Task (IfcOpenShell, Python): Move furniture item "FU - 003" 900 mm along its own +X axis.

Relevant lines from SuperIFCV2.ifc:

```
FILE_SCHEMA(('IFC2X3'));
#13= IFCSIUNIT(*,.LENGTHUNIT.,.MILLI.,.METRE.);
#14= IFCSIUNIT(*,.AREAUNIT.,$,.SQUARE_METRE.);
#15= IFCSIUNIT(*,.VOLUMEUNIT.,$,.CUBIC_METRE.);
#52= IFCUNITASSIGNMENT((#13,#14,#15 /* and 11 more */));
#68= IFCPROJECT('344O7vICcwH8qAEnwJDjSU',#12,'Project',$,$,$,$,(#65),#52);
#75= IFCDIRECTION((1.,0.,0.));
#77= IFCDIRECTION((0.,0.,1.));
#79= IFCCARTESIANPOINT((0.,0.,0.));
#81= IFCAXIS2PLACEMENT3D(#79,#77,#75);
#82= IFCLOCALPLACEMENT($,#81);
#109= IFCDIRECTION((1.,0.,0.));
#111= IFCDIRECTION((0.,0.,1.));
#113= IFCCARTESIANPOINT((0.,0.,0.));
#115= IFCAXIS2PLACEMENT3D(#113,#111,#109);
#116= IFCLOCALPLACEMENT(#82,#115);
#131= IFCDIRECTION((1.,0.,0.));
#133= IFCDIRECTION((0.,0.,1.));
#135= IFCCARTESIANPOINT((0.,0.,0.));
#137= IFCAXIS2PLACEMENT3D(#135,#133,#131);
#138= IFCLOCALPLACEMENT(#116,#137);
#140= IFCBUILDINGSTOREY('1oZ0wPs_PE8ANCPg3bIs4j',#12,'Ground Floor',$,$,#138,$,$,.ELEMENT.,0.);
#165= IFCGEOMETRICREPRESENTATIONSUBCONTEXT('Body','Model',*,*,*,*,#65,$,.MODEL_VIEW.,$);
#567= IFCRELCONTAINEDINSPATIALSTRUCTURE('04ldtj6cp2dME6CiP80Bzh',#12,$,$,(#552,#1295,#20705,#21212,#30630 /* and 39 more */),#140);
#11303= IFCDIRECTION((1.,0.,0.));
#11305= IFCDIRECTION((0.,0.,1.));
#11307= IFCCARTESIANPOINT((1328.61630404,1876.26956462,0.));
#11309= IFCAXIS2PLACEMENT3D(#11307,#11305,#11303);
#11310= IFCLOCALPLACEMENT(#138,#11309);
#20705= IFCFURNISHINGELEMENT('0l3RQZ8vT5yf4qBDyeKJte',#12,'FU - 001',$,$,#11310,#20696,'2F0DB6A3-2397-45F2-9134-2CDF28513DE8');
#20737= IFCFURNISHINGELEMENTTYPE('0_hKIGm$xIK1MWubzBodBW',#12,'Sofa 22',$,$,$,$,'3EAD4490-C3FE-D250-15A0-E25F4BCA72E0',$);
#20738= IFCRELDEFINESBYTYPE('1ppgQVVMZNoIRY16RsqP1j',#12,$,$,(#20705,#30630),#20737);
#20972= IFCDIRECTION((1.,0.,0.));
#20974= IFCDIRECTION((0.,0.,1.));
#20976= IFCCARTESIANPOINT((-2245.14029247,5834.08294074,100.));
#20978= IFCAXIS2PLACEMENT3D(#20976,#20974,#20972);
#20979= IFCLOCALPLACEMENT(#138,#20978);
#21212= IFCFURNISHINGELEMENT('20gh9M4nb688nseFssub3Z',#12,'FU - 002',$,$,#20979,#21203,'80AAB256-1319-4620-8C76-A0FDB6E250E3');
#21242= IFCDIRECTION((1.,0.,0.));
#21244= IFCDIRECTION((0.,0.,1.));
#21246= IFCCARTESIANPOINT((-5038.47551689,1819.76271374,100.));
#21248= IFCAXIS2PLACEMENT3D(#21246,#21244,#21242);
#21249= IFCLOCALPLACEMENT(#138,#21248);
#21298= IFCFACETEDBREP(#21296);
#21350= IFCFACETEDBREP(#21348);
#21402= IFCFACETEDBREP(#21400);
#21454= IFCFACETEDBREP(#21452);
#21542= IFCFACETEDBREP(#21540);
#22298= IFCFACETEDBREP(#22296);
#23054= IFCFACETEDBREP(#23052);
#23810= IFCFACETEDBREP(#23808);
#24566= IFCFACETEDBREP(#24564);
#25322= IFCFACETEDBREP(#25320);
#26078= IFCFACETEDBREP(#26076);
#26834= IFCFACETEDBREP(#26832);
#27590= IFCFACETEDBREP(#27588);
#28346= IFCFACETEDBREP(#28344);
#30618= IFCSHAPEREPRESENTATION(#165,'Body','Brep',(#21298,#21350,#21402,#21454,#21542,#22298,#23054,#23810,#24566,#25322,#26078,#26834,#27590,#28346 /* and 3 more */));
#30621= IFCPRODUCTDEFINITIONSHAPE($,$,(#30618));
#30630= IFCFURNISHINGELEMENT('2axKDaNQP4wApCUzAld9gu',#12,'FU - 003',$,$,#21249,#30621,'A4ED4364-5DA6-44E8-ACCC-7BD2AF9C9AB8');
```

```python
import ifcopenshell
import ifcopenshell.api.geometry
import ifcopenshell.util.placement

model = ifcopenshell.open("SuperIFCV2.ifc")

item = model.by_guid("2axKDaNQP4wApCUzAld9gu")
matrix = ifcopenshell.util.placement.get_local_placement(item.ObjectPlacement)
matrix[:3, 3] += matrix[:3, 0] * 900.0
ifcopenshell.api.geometry.edit_object_placement(model, product=item, matrix=matrix, is_si=False)

print(ifcopenshell.util.placement.get_local_placement(item.ObjectPlacement).round(3) + 0.0)

model.write("SuperIFCV2_edited.ifc")
```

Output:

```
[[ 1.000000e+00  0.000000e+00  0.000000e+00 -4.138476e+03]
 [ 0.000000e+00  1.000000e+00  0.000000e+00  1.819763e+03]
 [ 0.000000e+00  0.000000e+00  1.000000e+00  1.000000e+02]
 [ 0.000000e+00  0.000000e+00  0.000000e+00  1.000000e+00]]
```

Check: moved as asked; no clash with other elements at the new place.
